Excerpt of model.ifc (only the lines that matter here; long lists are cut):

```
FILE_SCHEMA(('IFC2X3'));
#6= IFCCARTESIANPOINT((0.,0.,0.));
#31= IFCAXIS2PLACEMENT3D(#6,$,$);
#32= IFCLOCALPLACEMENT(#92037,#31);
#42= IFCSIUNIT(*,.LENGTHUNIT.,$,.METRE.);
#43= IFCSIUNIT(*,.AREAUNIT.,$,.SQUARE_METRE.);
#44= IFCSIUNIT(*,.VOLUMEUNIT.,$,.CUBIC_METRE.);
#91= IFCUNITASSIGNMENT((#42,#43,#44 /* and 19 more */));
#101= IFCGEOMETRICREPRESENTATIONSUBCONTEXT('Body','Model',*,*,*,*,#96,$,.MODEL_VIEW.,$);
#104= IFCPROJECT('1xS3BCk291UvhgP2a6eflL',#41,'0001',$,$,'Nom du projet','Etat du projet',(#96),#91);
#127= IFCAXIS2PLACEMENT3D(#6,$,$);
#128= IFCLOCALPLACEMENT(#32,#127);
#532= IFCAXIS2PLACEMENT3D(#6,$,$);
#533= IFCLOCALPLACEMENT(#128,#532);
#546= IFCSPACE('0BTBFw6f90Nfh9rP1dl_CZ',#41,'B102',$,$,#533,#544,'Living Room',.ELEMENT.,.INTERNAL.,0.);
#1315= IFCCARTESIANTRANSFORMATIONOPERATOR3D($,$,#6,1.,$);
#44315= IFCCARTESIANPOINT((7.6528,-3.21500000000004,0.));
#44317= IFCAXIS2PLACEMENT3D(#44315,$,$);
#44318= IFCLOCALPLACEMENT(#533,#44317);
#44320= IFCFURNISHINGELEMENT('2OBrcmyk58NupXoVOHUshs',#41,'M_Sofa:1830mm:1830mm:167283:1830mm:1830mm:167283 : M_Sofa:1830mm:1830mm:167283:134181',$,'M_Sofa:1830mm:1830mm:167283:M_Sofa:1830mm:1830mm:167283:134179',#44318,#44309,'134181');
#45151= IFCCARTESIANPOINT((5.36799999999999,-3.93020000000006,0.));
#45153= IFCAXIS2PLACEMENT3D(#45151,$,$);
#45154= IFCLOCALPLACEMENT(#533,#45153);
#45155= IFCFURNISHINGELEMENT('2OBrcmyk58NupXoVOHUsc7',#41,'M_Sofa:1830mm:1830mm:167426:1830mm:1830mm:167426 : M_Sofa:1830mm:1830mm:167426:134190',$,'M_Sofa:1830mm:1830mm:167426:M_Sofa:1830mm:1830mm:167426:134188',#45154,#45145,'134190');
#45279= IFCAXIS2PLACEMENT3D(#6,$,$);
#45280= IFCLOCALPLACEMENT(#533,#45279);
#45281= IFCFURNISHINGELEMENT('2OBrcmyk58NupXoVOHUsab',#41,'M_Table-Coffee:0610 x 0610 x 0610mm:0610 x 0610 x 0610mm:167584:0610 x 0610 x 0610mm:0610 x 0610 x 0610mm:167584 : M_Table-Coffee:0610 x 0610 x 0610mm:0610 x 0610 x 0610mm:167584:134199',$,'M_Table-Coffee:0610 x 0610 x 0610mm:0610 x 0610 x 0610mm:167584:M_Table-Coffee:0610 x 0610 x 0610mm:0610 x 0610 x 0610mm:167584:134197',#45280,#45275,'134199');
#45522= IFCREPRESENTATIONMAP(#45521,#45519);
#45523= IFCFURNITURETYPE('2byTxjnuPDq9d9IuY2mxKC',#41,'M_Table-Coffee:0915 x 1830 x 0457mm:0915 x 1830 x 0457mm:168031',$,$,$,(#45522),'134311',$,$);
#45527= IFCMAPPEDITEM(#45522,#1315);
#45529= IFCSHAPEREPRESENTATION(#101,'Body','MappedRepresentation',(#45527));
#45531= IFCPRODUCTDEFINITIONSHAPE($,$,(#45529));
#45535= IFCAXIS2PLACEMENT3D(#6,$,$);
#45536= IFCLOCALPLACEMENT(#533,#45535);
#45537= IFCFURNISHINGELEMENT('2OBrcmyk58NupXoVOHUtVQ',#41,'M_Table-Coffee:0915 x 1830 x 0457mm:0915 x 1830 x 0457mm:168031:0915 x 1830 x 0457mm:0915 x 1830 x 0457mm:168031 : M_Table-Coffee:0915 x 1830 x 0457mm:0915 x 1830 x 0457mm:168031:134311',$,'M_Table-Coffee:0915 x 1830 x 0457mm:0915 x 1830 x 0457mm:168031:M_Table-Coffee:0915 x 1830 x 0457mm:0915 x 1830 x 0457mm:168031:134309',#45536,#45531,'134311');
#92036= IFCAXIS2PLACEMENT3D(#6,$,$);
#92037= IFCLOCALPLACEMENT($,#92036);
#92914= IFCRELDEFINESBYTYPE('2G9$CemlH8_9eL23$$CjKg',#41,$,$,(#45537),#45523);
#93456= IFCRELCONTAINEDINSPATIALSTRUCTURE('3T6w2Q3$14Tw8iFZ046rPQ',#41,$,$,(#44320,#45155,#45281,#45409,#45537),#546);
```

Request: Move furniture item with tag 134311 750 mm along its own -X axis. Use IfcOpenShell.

```python
import ifcopenshell
import ifcopenshell.api.geometry
import ifcopenshell.util.placement
import ifcopenshell.util.unit

model = ifcopenshell.open("model.ifc")
unit_scale = ifcopenshell.util.unit.calculate_unit_scale(model)

item = model.by_id(45537)
matrix = ifcopenshell.util.placement.get_local_placement(item.ObjectPlacement)
matrix[:3, 3] -= matrix[:3, 0] * 0.75 / unit_scale
ifcopenshell.api.geometry.edit_object_placement(model, product=item, matrix=matrix, is_si=False)

print(ifcopenshell.util.placement.get_local_placement(item.ObjectPlacement).round(3) + 0.0)

model.write("model_updated.ifc")
```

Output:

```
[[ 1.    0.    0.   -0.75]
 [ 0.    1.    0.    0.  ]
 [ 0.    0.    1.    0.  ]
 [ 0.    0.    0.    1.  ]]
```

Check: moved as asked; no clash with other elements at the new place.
